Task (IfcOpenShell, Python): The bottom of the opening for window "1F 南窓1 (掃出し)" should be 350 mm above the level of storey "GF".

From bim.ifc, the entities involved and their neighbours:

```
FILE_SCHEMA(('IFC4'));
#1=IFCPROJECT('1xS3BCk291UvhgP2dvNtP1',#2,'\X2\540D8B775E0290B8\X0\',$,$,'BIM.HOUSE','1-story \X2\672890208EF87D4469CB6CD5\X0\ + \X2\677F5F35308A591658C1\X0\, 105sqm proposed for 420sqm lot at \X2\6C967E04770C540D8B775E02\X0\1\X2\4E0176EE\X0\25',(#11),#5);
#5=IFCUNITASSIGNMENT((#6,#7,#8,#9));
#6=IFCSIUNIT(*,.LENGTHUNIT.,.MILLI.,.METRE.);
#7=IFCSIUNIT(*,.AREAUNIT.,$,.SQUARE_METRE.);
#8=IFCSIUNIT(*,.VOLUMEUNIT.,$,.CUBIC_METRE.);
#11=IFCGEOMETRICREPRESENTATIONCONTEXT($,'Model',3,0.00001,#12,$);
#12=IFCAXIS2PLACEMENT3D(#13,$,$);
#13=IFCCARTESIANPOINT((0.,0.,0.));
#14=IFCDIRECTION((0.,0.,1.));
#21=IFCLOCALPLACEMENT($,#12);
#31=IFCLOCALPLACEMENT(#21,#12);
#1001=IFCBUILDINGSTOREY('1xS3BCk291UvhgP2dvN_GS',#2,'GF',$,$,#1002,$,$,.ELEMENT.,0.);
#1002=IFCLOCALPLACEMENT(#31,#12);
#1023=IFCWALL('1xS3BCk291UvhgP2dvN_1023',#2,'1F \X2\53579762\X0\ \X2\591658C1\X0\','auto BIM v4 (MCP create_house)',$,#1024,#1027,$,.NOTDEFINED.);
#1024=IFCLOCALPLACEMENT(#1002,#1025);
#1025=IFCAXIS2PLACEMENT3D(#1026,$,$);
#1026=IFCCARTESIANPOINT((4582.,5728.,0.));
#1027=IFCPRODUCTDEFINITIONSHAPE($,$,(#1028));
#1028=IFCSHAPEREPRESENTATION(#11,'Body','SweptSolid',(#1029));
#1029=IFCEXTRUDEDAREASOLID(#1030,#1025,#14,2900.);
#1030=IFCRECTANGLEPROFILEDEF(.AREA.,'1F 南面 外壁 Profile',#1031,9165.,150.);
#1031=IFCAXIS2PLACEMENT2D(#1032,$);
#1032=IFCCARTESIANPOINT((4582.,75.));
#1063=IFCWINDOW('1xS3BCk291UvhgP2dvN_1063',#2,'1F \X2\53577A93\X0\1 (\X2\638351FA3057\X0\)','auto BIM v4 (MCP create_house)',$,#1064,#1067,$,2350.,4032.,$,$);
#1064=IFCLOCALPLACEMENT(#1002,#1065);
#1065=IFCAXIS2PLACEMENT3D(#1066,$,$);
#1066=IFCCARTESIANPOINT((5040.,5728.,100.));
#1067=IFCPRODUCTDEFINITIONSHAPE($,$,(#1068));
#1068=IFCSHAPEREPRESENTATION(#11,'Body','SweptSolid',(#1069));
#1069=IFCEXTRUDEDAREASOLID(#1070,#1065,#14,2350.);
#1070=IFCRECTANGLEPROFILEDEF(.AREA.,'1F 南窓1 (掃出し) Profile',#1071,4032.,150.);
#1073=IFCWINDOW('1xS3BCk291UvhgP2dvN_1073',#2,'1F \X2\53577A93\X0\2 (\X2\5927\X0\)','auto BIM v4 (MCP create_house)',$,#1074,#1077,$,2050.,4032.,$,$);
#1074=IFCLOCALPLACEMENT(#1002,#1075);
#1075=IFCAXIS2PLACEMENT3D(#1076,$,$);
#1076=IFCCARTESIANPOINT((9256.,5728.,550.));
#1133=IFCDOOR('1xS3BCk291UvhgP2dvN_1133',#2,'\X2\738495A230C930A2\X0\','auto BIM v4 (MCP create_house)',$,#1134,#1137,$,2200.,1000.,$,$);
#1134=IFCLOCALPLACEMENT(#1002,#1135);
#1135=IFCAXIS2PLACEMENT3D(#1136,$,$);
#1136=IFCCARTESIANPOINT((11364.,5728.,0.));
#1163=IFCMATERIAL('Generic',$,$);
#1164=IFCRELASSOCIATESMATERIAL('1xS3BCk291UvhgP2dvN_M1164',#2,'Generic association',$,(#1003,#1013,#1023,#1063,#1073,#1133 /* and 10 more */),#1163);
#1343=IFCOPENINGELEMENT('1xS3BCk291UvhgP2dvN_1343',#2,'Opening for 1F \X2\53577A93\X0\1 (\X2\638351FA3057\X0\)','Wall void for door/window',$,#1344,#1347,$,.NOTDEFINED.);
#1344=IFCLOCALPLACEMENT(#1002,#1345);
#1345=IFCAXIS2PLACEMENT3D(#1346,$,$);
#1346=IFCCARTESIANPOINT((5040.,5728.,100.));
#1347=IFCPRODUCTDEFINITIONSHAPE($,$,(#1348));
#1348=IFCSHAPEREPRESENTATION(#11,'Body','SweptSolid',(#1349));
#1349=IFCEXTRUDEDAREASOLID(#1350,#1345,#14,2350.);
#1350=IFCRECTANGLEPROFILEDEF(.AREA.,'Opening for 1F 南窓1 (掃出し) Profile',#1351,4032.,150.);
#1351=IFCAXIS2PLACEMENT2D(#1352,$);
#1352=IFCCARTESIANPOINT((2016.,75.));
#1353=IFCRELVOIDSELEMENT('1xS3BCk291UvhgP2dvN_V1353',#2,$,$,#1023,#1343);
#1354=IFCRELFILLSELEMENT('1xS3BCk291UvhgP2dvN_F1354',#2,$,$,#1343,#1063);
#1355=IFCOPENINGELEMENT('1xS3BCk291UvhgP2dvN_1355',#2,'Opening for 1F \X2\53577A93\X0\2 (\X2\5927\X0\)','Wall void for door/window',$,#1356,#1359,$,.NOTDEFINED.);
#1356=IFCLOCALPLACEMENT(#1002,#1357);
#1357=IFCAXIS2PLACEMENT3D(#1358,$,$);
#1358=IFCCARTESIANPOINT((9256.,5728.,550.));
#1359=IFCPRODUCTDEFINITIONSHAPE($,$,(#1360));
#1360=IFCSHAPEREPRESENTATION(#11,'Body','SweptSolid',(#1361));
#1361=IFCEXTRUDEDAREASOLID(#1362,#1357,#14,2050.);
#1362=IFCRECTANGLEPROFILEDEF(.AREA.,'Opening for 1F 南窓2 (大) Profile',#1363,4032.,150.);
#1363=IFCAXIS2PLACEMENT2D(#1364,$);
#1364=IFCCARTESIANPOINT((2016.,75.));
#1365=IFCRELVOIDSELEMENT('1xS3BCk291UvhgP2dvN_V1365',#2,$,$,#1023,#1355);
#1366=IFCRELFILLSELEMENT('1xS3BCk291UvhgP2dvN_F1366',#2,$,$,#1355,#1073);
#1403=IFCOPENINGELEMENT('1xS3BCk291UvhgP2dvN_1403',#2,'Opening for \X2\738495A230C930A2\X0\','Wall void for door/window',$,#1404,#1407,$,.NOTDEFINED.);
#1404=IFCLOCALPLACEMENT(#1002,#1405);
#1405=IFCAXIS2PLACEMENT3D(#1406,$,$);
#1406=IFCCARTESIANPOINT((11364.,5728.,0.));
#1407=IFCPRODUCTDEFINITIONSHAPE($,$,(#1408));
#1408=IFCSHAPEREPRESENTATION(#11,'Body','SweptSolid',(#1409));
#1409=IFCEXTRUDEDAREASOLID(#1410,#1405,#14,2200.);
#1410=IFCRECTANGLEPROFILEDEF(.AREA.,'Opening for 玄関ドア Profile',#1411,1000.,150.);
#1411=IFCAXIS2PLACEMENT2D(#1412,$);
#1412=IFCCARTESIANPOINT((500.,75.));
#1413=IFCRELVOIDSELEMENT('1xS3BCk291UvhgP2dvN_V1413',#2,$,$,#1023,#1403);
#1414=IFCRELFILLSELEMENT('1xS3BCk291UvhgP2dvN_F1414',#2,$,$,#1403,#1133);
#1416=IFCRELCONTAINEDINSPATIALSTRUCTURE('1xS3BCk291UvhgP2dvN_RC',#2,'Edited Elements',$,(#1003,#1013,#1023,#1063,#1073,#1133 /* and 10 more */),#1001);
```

```python
import numpy as np
import ifcopenshell
import ifcopenshell.api.geometry
import ifcopenshell.geom
import ifcopenshell.util.element
import ifcopenshell.util.placement
import ifcopenshell.util.shape
import ifcopenshell.util.unit

model = ifcopenshell.open("bim.ifc")
unit_scale = ifcopenshell.util.unit.calculate_unit_scale(model)

window = model.by_guid("1xS3BCk291UvhgP2dvN_1063")
opening = window.FillsVoids[0].RelatingOpeningElement
storey = ifcopenshell.util.element.get_container(window, ifc_class="IfcBuildingStorey")
level = ifcopenshell.util.placement.get_local_placement(storey.ObjectPlacement)[2, 3]

# The opening's origin need not be at the sill, so measure its lowest point.
shape = ifcopenshell.geom.create_shape(ifcopenshell.geom.settings(), opening)
bottom = ifcopenshell.util.shape.get_shape_bottom_elevation(shape, shape.geometry) / unit_scale
dz = level + 0.35 / unit_scale - bottom

shift = np.array([0.0, 0.0, dz])
# The window is not placed relative to its opening, so move both.
for product in (opening, window):
    matrix = ifcopenshell.util.placement.get_local_placement(product.ObjectPlacement)
    matrix[:3, 3] += shift
    ifcopenshell.api.geometry.edit_object_placement(model, product=product, matrix=matrix, is_si=False)

print(f"moved by {dz * unit_scale:+.3f} m")

model.write("bim-out.ifc")
```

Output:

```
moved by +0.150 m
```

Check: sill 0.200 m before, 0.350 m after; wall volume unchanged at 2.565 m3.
